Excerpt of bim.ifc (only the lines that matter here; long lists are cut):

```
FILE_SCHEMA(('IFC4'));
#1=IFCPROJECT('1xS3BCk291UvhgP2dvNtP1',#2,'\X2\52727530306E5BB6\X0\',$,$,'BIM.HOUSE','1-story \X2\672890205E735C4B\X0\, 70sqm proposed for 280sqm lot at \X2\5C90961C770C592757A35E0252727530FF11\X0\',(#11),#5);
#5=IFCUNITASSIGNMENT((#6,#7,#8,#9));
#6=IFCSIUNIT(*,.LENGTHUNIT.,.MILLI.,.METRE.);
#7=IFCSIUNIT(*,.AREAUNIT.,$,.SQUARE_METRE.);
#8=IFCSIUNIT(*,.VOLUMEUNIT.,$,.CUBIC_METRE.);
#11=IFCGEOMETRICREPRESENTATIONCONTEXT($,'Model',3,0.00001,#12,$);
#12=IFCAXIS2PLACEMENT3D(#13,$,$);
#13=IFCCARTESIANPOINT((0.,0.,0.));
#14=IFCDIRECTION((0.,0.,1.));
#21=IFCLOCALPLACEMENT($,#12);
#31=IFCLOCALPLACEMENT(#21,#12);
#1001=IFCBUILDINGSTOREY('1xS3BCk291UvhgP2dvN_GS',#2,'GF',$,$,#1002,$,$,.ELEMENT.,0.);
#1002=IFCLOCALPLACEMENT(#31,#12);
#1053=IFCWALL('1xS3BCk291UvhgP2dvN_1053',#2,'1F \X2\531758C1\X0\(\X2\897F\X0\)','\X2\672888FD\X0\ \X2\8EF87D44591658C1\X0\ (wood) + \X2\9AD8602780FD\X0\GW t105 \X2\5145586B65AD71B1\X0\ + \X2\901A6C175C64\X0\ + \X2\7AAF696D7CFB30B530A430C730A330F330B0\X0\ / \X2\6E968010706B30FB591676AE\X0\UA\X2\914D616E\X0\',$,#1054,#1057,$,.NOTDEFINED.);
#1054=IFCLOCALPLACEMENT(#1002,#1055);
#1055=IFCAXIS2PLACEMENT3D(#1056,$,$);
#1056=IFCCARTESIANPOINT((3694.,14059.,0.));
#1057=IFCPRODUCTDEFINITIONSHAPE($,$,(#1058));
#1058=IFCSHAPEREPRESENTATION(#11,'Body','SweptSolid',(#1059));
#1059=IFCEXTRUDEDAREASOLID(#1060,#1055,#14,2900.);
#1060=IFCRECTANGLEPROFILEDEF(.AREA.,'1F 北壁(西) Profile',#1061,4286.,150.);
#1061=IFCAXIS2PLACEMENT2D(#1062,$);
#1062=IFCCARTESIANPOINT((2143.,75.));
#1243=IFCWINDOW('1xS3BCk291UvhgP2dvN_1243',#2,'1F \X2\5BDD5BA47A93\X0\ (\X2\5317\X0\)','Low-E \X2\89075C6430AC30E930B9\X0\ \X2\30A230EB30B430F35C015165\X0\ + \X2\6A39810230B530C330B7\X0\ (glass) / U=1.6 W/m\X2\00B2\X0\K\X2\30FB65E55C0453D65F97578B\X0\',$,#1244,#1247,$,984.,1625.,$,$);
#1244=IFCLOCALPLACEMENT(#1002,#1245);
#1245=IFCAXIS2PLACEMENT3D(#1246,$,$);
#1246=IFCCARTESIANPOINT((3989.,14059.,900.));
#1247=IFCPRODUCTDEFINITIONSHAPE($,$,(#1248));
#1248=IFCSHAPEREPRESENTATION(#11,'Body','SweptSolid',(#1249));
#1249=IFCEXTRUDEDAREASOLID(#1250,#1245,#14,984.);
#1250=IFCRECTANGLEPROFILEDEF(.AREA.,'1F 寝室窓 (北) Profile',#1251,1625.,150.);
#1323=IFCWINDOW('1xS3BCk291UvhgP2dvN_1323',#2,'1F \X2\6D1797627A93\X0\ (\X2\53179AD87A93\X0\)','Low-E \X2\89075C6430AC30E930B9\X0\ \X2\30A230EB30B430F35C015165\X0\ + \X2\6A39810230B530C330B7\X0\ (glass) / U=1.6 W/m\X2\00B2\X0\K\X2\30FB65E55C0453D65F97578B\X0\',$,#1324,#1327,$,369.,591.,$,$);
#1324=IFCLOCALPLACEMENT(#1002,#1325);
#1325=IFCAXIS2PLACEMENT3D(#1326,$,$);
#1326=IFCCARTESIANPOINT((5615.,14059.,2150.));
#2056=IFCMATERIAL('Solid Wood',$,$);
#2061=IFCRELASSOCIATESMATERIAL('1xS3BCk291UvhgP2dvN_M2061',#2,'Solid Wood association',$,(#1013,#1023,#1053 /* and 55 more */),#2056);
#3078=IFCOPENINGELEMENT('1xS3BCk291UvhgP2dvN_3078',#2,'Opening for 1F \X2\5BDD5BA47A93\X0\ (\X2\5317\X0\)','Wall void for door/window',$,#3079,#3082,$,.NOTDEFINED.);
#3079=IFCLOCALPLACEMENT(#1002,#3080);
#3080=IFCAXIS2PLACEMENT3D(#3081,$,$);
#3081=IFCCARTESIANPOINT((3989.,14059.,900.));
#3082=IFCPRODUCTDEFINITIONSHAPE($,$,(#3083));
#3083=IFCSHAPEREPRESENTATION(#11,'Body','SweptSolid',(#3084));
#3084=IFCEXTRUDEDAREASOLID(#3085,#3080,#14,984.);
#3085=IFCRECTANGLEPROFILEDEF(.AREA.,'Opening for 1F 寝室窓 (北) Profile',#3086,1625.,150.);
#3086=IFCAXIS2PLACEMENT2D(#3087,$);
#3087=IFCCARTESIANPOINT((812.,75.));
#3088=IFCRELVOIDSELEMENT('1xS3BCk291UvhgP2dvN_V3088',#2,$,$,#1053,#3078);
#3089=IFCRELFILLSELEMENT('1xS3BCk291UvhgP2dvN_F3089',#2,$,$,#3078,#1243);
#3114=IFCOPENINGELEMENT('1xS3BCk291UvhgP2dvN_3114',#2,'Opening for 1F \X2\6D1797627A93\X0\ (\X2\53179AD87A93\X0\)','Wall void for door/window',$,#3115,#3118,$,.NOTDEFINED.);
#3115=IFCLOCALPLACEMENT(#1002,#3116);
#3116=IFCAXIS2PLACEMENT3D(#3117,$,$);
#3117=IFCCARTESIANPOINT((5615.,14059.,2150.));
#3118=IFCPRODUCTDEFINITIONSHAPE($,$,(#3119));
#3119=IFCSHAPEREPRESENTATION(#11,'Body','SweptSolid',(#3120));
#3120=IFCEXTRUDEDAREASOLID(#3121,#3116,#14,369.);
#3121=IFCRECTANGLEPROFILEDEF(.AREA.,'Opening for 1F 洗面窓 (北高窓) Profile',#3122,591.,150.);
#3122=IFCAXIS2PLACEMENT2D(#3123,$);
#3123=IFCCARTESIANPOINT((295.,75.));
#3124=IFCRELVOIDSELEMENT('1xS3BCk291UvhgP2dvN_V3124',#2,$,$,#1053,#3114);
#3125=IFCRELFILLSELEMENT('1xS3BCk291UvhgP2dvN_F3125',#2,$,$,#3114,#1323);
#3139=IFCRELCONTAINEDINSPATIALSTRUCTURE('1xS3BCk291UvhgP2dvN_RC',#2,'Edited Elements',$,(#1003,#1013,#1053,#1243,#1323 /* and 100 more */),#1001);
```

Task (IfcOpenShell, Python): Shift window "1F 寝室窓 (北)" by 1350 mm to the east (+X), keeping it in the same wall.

```python
import ifcopenshell
import ifcopenshell.api.geometry
import ifcopenshell.util.placement

model = ifcopenshell.open("bim.ifc")

window = model.by_id(1243)
opening = window.FillsVoids[0].RelatingOpeningElement
wall = opening.VoidsElements[0].RelatingBuildingElement

wall_matrix = ifcopenshell.util.placement.get_local_placement(wall.ObjectPlacement)
shift = wall_matrix[:3, 0] * 1350.0
before = ifcopenshell.util.placement.get_local_placement(window.ObjectPlacement)[:3, 3].copy()

# The window is not placed relative to its opening, so move both.
for product in (opening, window):
    matrix = ifcopenshell.util.placement.get_local_placement(product.ObjectPlacement)
    matrix[:3, 3] += shift
    ifcopenshell.api.geometry.edit_object_placement(model, product=product, matrix=matrix, is_si=False)

after = ifcopenshell.util.placement.get_local_placement(window.ObjectPlacement)[:3, 3]
print("window moved by", (after - before).round(3) + 0.0)

model.write("bim-out.ifc")
```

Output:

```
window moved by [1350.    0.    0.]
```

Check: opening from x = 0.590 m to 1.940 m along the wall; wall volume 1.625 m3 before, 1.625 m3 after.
